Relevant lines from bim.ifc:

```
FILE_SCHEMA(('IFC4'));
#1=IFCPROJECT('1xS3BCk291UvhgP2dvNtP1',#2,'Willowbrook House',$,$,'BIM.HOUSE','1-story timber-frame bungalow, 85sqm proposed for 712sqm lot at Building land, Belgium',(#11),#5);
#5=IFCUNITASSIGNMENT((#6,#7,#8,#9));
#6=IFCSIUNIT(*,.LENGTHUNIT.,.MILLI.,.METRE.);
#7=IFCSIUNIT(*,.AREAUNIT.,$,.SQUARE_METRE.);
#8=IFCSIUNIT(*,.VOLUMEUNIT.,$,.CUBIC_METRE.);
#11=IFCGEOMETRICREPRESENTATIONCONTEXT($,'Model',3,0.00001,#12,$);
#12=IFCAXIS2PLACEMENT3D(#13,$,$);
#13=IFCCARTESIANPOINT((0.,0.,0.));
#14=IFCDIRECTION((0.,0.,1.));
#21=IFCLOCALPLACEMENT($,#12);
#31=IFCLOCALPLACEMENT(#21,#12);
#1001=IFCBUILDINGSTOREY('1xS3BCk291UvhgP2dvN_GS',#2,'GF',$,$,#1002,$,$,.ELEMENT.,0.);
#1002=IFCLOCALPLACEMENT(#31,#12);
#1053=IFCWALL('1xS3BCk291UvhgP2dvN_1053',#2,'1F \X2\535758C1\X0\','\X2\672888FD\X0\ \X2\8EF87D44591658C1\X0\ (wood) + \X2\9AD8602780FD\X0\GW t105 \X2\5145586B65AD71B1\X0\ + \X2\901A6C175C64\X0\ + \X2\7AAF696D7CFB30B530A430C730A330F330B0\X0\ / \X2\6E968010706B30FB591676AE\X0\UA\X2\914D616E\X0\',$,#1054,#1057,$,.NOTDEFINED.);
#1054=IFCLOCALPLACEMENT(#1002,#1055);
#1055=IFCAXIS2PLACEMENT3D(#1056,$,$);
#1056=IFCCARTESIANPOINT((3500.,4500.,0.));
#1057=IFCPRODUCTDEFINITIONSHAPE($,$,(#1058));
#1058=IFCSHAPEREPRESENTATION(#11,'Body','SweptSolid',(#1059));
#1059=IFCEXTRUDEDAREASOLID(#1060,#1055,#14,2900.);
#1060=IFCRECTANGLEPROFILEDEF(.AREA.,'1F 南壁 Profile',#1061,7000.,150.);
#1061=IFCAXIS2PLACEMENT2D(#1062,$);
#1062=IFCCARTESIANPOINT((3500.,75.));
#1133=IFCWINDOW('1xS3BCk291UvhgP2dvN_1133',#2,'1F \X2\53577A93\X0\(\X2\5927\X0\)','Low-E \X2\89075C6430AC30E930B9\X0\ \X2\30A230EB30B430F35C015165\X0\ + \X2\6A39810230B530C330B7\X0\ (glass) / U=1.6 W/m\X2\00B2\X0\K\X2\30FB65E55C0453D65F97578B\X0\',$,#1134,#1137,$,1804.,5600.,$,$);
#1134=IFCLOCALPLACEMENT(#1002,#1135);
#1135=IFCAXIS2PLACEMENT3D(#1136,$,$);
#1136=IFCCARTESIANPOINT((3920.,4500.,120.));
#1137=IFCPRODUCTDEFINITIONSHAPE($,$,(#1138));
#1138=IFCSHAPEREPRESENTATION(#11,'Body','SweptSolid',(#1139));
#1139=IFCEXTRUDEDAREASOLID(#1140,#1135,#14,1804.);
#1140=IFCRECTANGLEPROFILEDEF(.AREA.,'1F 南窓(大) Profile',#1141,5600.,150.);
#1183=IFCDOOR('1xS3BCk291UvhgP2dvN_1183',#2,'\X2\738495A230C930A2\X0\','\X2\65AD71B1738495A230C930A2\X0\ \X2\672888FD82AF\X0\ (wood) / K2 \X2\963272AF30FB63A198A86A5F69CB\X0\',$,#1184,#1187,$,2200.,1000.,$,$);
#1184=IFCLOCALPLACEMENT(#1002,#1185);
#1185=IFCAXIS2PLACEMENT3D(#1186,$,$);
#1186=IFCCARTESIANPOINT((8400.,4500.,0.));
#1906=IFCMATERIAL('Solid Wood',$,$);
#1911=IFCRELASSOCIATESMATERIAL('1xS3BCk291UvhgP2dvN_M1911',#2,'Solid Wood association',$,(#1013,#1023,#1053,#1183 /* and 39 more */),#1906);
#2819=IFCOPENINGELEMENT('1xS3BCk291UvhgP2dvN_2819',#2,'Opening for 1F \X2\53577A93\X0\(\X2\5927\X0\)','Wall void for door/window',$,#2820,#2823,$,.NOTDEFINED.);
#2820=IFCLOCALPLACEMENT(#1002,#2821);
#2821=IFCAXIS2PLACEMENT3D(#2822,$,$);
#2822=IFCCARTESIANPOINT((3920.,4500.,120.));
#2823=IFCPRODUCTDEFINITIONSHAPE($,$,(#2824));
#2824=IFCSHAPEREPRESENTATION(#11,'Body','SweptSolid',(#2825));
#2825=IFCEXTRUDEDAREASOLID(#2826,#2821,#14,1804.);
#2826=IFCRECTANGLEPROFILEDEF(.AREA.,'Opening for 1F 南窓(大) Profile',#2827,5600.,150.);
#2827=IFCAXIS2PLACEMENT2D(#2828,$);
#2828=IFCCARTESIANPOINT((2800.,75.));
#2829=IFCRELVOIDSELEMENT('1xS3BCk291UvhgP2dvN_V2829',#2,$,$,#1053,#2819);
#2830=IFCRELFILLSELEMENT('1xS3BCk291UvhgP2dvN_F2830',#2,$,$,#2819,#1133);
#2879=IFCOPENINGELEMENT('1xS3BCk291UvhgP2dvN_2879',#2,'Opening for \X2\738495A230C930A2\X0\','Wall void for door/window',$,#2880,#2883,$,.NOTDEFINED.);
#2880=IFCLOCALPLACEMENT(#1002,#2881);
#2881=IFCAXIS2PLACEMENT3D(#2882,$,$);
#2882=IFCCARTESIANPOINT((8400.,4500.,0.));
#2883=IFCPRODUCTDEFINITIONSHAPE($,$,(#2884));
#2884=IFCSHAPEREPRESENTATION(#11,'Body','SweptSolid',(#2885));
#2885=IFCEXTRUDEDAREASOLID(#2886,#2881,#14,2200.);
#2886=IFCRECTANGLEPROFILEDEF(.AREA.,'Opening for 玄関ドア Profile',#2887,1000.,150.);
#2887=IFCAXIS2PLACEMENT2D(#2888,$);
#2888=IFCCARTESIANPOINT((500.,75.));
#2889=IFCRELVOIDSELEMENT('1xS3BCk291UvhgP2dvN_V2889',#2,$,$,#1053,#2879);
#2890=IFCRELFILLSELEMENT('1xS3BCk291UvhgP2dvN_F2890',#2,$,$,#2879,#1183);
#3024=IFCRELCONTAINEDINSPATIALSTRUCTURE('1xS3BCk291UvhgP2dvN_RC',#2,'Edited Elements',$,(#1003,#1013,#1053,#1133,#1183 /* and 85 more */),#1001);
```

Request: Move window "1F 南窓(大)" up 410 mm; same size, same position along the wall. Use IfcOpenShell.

```python
import numpy as np
import ifcopenshell
import ifcopenshell.api.geometry
import ifcopenshell.util.placement
import ifcopenshell.util.unit

model = ifcopenshell.open("bim.ifc")
unit_scale = ifcopenshell.util.unit.calculate_unit_scale(model)

window = model.by_id(1133)
opening = window.FillsVoids[0].RelatingOpeningElement
dz = 0.41 / unit_scale

shift = np.array([0.0, 0.0, dz])
# The window is not placed relative to its opening, so move both.
for product in (opening, window):
    matrix = ifcopenshell.util.placement.get_local_placement(product.ObjectPlacement)
    matrix[:3, 3] += shift
    ifcopenshell.api.geometry.edit_object_placement(model, product=product, matrix=matrix, is_si=False)

print(f"moved by {dz * unit_scale:+.3f} m")

model.write("bim-out.ifc")
```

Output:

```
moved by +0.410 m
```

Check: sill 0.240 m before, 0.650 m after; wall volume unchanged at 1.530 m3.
